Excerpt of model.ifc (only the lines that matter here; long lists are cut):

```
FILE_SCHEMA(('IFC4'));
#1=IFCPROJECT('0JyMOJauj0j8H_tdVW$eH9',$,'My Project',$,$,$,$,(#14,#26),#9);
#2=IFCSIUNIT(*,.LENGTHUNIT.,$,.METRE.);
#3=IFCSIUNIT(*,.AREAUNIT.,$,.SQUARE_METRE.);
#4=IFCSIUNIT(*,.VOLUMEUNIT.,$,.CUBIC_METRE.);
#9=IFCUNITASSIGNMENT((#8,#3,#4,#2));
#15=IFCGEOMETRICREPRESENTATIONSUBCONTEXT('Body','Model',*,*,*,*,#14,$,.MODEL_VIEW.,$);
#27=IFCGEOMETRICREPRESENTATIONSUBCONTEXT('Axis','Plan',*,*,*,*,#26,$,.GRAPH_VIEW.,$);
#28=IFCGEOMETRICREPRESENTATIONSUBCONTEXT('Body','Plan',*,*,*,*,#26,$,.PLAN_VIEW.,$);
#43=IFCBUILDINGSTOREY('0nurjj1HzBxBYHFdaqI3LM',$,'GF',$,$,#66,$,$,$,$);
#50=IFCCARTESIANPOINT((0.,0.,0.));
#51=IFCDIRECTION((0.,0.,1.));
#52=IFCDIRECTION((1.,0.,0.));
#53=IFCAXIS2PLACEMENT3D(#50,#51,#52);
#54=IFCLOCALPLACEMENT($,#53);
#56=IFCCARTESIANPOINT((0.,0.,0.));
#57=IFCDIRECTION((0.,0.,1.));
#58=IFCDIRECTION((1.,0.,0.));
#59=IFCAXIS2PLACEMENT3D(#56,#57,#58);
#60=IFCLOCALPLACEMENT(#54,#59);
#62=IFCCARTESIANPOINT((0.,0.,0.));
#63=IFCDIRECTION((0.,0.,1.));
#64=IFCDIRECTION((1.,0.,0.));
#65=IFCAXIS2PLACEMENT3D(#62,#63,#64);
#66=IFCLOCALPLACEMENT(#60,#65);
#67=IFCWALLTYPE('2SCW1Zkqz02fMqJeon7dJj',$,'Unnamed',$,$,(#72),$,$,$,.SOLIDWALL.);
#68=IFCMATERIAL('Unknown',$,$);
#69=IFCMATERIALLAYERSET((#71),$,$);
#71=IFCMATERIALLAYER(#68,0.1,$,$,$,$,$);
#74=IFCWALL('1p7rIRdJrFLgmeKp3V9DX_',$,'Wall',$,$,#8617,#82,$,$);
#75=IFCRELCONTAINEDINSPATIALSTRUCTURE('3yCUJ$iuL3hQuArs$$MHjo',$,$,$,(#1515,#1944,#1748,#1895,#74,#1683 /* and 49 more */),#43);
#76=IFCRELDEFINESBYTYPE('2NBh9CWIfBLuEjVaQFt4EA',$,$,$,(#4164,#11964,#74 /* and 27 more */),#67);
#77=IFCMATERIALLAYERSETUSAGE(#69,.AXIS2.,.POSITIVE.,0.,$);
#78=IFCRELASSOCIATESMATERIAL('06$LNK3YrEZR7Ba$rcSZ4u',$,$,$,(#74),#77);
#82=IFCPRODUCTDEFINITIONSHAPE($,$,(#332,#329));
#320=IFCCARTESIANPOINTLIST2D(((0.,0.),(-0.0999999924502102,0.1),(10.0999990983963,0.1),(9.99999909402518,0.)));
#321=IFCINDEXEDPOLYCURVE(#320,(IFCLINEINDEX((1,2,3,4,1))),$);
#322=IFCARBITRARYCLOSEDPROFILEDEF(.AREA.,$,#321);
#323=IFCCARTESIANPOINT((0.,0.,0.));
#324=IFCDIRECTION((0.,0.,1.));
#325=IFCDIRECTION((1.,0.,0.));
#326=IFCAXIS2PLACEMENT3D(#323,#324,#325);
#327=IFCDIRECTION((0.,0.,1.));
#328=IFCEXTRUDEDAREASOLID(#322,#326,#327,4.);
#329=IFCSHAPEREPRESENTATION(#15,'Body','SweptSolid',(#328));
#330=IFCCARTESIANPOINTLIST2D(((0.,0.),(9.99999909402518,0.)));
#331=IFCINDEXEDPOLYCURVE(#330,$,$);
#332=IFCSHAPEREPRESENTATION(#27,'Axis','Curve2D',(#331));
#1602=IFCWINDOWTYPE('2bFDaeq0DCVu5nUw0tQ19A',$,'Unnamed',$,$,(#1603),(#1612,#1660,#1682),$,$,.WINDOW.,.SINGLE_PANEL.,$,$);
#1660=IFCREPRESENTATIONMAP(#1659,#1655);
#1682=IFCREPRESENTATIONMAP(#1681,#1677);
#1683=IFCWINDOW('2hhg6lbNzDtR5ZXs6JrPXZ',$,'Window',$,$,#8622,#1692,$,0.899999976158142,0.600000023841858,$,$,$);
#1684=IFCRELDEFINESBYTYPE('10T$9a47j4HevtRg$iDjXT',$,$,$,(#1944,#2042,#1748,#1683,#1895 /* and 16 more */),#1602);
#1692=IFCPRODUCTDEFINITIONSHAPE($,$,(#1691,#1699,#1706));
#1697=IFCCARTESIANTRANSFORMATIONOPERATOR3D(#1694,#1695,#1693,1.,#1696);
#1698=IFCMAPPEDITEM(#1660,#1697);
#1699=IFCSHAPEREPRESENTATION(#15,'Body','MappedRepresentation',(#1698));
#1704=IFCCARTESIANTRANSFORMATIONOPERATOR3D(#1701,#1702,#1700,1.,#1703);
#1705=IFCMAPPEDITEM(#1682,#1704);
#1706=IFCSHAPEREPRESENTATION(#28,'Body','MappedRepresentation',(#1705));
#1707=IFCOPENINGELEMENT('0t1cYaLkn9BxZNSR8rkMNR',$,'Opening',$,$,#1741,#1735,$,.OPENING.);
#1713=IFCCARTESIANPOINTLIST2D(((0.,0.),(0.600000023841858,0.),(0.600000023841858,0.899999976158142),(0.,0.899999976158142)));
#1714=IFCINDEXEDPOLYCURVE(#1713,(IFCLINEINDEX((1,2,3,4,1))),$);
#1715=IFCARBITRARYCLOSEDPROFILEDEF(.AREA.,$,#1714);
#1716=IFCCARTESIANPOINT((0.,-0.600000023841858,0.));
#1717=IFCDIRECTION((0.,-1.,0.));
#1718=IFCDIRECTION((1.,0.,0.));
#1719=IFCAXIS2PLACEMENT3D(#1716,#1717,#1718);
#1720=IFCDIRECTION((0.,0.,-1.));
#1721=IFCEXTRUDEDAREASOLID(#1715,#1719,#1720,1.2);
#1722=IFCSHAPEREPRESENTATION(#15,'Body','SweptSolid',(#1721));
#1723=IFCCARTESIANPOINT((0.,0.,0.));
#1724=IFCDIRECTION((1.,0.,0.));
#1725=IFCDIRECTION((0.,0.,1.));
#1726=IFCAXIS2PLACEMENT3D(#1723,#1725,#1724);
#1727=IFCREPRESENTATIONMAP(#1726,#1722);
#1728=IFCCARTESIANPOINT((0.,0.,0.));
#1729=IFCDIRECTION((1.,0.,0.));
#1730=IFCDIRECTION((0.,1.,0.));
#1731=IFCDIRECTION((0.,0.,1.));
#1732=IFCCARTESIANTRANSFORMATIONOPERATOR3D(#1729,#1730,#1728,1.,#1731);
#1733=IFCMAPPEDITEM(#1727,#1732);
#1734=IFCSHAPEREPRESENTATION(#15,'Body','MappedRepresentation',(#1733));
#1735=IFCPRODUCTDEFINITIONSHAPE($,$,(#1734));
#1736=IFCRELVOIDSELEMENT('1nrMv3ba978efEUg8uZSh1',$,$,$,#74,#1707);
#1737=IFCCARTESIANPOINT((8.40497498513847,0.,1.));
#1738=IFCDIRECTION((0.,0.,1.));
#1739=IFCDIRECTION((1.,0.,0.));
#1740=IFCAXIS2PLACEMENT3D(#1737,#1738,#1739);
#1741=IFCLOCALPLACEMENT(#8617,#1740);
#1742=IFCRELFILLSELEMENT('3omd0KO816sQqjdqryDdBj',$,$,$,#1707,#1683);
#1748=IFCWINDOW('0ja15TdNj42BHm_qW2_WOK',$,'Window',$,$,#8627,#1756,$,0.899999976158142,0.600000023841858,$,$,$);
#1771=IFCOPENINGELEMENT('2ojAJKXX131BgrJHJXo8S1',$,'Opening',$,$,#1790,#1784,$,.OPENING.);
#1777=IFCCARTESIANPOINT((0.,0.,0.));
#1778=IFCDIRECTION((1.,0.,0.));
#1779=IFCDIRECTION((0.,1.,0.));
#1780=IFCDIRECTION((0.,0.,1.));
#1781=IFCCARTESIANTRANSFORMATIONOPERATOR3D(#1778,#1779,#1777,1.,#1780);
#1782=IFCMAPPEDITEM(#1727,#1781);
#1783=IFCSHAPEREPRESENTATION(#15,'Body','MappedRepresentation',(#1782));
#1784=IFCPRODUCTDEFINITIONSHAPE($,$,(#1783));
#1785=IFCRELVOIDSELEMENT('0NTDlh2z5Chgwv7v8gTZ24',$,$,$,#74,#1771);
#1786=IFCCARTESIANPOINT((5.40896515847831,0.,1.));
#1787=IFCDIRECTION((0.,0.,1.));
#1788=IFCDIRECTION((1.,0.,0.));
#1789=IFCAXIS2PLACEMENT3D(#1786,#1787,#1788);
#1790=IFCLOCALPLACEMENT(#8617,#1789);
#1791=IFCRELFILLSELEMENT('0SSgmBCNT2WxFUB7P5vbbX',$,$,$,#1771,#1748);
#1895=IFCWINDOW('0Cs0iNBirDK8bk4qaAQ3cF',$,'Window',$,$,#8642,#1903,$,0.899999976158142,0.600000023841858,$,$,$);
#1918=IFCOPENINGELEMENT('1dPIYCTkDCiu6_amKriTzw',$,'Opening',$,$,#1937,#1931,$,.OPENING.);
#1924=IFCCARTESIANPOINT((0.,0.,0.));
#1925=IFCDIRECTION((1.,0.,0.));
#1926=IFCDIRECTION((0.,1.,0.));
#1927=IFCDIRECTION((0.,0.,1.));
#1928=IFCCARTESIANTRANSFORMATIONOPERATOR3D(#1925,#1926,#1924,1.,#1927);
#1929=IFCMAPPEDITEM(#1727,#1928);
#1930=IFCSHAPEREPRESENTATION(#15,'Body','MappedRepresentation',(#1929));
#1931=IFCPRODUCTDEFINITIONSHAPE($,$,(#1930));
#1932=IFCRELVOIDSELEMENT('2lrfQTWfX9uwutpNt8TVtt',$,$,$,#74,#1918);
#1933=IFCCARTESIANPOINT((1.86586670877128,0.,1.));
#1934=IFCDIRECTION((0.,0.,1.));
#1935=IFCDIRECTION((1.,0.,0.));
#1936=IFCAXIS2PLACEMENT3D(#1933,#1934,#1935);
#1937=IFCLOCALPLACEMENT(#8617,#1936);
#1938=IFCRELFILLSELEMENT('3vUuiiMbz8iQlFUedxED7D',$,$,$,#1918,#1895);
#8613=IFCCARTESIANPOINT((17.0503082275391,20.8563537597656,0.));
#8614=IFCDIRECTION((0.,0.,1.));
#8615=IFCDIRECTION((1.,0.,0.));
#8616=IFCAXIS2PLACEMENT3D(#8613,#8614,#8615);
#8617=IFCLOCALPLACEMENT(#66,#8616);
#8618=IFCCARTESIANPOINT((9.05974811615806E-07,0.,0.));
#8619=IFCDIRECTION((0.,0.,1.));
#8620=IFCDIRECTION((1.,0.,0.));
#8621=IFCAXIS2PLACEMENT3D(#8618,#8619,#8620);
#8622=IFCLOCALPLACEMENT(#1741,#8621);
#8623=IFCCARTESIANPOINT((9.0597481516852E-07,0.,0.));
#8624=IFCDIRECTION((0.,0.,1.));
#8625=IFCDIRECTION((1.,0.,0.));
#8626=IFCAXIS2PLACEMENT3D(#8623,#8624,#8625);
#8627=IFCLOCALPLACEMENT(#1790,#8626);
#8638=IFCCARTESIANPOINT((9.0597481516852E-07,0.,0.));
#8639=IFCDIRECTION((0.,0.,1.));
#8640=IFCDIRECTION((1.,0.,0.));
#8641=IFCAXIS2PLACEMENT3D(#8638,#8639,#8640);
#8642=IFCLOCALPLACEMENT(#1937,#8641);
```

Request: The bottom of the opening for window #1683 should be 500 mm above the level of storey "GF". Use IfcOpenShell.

```python
import numpy as np
import ifcopenshell
import ifcopenshell.api.geometry
import ifcopenshell.geom
import ifcopenshell.util.element
import ifcopenshell.util.placement
import ifcopenshell.util.shape
import ifcopenshell.util.unit

model = ifcopenshell.open("model.ifc")
unit_scale = ifcopenshell.util.unit.calculate_unit_scale(model)

window = model.by_guid("2hhg6lbNzDtR5ZXs6JrPXZ")
opening = window.FillsVoids[0].RelatingOpeningElement
storey = ifcopenshell.util.element.get_container(window, ifc_class="IfcBuildingStorey")
level = ifcopenshell.util.placement.get_local_placement(storey.ObjectPlacement)[2, 3]

# The opening's origin need not be at the sill, so measure its lowest point.
shape = ifcopenshell.geom.create_shape(ifcopenshell.geom.settings(), opening)
bottom = ifcopenshell.util.shape.get_shape_bottom_elevation(shape, shape.geometry) / unit_scale
dz = level + 0.5 / unit_scale - bottom

shift = np.array([0.0, 0.0, dz])
# The window is placed relative to its opening, so it follows when the opening moves.
matrix = ifcopenshell.util.placement.get_local_placement(opening.ObjectPlacement)
matrix[:3, 3] += shift
ifcopenshell.api.geometry.edit_object_placement(
    model, product=opening, matrix=matrix, is_si=False, should_transform_children=True
)

print(f"moved by {dz * unit_scale:+.3f} m")

model.write("model_v2.ifc")
```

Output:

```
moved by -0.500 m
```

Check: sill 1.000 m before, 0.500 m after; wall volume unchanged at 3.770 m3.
